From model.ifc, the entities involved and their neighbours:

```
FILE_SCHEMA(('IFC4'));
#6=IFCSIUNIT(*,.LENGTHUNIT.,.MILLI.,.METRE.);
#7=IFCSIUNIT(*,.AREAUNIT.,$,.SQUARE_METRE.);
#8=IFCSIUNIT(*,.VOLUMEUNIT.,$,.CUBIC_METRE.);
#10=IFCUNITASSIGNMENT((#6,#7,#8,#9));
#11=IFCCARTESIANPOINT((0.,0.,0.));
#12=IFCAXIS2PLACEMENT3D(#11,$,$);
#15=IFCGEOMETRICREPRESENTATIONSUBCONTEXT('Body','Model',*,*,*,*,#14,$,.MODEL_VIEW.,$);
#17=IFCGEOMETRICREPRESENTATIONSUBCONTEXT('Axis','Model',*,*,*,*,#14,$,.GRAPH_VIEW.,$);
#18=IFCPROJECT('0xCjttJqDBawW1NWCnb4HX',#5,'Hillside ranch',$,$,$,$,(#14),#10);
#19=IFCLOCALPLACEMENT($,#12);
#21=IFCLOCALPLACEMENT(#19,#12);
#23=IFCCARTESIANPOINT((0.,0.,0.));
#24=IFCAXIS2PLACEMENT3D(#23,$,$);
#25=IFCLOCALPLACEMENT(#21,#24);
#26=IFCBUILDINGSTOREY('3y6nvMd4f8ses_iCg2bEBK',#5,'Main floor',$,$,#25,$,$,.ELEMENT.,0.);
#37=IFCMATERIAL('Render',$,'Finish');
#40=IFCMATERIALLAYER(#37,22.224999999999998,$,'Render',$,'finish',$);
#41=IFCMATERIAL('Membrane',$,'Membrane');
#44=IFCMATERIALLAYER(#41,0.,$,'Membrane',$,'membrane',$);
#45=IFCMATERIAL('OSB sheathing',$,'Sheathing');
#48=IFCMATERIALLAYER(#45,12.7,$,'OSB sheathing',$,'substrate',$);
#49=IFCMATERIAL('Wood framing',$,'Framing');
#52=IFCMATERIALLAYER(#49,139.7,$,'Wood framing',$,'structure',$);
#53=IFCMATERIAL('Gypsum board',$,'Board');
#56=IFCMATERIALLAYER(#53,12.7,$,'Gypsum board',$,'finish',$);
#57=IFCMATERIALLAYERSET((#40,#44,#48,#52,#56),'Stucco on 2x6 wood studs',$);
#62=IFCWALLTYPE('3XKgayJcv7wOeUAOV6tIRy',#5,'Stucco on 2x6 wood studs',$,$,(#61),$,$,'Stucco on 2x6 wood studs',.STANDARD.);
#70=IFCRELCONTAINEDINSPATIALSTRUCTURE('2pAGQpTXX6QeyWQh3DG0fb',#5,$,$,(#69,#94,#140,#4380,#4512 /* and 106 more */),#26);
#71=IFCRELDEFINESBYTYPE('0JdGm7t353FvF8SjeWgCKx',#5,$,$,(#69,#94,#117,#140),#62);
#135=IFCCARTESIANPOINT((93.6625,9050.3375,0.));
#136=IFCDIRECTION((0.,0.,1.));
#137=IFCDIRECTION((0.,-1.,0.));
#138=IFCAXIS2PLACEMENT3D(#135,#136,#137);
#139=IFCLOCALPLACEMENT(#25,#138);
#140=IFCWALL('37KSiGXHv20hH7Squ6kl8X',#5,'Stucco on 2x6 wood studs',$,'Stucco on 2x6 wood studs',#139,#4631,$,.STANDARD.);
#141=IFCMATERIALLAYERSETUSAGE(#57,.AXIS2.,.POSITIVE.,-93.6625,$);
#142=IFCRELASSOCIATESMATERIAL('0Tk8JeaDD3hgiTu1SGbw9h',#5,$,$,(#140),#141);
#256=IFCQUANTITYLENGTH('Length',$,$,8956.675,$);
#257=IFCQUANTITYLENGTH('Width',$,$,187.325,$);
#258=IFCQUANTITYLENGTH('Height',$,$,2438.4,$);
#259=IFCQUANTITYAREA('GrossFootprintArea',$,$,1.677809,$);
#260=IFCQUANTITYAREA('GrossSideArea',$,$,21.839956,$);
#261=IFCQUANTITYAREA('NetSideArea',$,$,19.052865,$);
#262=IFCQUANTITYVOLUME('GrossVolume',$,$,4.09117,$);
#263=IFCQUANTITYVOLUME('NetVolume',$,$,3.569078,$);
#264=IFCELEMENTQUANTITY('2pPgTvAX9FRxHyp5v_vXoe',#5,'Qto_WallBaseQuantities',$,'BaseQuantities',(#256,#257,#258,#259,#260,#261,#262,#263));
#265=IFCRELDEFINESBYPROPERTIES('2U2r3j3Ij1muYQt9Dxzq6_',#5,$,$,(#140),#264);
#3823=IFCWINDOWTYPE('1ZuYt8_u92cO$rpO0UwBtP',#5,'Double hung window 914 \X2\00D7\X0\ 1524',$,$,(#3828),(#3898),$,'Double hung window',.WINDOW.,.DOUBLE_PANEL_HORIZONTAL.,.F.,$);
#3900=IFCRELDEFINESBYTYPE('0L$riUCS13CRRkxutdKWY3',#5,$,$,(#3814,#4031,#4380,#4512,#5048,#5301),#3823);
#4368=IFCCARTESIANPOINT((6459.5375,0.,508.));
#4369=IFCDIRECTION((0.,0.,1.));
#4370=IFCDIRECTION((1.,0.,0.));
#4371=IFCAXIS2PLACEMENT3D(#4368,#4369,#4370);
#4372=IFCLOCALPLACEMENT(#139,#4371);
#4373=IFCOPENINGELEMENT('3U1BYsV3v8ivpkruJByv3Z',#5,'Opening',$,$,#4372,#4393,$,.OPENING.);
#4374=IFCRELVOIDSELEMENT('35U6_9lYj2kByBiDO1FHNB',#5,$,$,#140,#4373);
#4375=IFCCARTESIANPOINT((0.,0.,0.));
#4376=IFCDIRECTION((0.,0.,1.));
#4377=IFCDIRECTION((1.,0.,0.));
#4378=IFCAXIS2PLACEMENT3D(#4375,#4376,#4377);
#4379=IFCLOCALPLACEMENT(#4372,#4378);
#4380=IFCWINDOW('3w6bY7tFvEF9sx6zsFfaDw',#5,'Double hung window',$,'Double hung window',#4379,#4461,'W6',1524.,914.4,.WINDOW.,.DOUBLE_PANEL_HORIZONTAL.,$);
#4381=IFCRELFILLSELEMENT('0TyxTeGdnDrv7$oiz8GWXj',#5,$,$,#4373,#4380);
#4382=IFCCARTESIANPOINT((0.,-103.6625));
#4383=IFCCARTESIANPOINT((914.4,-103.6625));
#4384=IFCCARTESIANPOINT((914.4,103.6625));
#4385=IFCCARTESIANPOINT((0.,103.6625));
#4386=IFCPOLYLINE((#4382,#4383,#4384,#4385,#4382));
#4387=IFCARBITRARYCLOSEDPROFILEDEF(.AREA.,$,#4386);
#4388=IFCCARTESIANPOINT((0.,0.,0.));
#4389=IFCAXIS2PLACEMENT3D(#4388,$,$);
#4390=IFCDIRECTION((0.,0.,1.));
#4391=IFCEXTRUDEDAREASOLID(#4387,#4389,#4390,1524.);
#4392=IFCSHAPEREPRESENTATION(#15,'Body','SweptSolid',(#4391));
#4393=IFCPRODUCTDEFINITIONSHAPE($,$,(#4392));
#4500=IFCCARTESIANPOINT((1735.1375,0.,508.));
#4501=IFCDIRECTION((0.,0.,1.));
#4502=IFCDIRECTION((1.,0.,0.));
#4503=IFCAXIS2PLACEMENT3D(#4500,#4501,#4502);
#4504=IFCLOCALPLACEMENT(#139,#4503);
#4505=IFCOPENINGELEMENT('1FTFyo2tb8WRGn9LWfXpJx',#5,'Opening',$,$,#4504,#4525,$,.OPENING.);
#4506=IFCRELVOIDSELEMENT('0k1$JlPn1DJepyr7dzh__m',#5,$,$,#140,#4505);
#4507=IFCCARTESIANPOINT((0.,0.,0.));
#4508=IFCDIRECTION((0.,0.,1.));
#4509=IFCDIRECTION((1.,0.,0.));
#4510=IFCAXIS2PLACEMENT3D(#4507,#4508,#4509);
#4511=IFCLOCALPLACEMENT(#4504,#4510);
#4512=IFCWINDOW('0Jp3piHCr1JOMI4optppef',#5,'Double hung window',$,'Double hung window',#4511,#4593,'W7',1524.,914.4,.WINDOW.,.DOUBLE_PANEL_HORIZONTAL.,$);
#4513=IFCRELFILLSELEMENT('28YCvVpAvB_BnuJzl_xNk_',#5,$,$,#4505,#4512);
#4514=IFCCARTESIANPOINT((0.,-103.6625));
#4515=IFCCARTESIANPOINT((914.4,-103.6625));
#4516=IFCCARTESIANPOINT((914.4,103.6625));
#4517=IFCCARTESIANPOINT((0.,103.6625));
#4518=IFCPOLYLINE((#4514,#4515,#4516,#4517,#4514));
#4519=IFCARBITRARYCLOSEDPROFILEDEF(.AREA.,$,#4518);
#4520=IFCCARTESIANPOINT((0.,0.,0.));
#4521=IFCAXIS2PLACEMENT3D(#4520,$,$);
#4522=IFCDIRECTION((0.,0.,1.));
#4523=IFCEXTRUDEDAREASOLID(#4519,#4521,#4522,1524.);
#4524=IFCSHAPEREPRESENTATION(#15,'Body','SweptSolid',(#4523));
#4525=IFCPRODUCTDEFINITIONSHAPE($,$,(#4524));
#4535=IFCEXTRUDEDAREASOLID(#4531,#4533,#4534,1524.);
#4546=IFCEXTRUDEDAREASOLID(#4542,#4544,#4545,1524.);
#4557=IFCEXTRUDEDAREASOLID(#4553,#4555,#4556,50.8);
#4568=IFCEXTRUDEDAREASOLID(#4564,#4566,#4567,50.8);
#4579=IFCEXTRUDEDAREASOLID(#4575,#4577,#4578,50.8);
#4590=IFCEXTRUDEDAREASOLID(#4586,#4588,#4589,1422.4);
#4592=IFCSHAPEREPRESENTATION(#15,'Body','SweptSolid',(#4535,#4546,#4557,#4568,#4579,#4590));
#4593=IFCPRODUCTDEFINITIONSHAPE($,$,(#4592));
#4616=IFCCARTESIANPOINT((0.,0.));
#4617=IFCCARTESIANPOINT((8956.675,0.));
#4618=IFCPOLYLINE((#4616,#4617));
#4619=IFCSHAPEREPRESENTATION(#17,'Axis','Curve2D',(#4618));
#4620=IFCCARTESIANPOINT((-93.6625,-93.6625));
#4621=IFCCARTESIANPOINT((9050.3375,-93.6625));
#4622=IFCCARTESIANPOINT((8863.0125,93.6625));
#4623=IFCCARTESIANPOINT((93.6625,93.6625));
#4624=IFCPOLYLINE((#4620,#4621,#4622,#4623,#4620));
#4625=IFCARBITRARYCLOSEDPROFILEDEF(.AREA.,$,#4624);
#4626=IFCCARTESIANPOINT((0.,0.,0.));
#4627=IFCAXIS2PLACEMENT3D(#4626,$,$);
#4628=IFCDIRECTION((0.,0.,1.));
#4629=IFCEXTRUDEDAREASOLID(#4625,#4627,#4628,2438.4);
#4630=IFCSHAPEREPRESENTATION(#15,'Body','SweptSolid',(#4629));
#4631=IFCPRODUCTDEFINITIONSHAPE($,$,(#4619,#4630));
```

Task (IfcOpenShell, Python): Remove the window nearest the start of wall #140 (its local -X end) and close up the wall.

```python
import ifcopenshell
import ifcopenshell.api.feature
import ifcopenshell.api.pset
import ifcopenshell.api.root
import ifcopenshell.geom
import ifcopenshell.util.element
import ifcopenshell.util.shape
import ifcopenshell.util.unit

model = ifcopenshell.open("model.ifc")
area_scale = ifcopenshell.util.unit.calculate_unit_scale(model, "AREAUNIT")
volume_scale = ifcopenshell.util.unit.calculate_unit_scale(model, "VOLUMEUNIT")
settings = ifcopenshell.geom.settings()


def volume(element):
    """Net volume in cubic metres, openings subtracted."""
    shape = ifcopenshell.geom.create_shape(settings, element)
    return ifcopenshell.util.shape.get_volume(shape.geometry)


window = model.by_id(4512)
opening = window.FillsVoids[0].RelatingOpeningElement
wall = opening.VoidsElements[0].RelatingBuildingElement
before = volume(wall)

ifcopenshell.api.root.remove_product(model, product=window)
ifcopenshell.api.feature.remove_feature(model, feature=opening)

after = volume(wall)
thickness = 0.1873  # wall thickness in metres

# Update the wall's stored quantities.
qto = model.by_id(ifcopenshell.util.element.get_pset(wall, "Qto_WallBaseQuantities", should_inherit=False)["id"])
ifcopenshell.api.pset.edit_qto(model, qto=qto, properties={
    "NetSideArea": after / thickness / area_scale,
    "NetVolume": after / volume_scale,
})

print(f"wall volume {before:.3f} -> {after:.3f} m3")

model.write("model_updated.ifc")
```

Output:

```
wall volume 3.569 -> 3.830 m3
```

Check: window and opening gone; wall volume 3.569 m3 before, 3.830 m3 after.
